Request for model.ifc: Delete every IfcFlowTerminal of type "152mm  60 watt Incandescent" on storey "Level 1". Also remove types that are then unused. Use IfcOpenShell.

First a look at what the model holds.

```python
import ifcopenshell
import ifcopenshell.util.element

model = ifcopenshell.open("model.ifc")
print(model.schema)
storey = next(s for s in model.by_type("IfcBuildingStorey") if s.Name == "Level 1")
terminals = [e for e in ifcopenshell.util.element.get_decomposition(storey) if e.is_a("IfcFlowTerminal")]
seen = {}
for e in terminals:
    element_type = ifcopenshell.util.element.get_type(e)
    name = element_type.Name if element_type not in (None, e) else None
    seen[name] = seen.get(name, 0) + 1
for name, count in sorted(seen.items(), key=str):
    print(count, "x", name)
```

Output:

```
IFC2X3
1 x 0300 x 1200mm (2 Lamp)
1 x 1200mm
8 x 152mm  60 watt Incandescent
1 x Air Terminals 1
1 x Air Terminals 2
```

```python
import ifcopenshell
import ifcopenshell.api.root
import ifcopenshell.util.element

model = ifcopenshell.open("model.ifc")

storey = next(s for s in model.by_type("IfcBuildingStorey") if s.Name == "Level 1")
terminals = [e for e in ifcopenshell.util.element.get_decomposition(storey) if e.is_a("IfcFlowTerminal")]
targets = [e for e in terminals if (t := ifcopenshell.util.element.get_type(e)) not in (None, e) and t.Name == "152mm  60 watt Incandescent"]
types = {ifcopenshell.util.element.get_type(e) for e in targets} - {None, *targets}

for e in targets:
    ifcopenshell.api.root.remove_product(model, product=e)
print(len(targets), "removed")

unused = [t for t in types if not ifcopenshell.util.element.get_types(t)]
for t in unused:
    ifcopenshell.api.root.remove_product(model, product=t)
print(len(unused), "unused types removed")

model.write("model-out.ifc")
```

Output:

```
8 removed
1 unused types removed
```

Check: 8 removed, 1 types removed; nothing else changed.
